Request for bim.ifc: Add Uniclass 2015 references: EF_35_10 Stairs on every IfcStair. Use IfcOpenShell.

First a look at what the model holds.

```python
import ifcopenshell

model = ifcopenshell.open("bim.ifc")
print(model.schema)
print("classifications:", [c.Name for c in model.by_type("IfcClassification")])
for ifc_class in ("IfcDoor", "IfcRoof", "IfcStair", "IfcWall", "IfcWindow"):
    print(ifc_class, len(model.by_type(ifc_class)))
```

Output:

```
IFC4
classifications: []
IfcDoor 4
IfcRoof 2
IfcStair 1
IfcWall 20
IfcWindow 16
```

```python
import ifcopenshell
import ifcopenshell.api.classification

model = ifcopenshell.open("bim.ifc")

system = ifcopenshell.api.classification.add_classification(model, classification="Uniclass 2015")

codes = {
    "IfcStair": ("EF_35_10", "Stairs"),
}
for ifc_class, (code, name) in codes.items():
    products = model.by_type(ifc_class)
    ifcopenshell.api.classification.add_reference(
        model, products=products, classification=system, identification=code, name=name
    )
    print(code, len(products))

model.write("bim-out.ifc")
```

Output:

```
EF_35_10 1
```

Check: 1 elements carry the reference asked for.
